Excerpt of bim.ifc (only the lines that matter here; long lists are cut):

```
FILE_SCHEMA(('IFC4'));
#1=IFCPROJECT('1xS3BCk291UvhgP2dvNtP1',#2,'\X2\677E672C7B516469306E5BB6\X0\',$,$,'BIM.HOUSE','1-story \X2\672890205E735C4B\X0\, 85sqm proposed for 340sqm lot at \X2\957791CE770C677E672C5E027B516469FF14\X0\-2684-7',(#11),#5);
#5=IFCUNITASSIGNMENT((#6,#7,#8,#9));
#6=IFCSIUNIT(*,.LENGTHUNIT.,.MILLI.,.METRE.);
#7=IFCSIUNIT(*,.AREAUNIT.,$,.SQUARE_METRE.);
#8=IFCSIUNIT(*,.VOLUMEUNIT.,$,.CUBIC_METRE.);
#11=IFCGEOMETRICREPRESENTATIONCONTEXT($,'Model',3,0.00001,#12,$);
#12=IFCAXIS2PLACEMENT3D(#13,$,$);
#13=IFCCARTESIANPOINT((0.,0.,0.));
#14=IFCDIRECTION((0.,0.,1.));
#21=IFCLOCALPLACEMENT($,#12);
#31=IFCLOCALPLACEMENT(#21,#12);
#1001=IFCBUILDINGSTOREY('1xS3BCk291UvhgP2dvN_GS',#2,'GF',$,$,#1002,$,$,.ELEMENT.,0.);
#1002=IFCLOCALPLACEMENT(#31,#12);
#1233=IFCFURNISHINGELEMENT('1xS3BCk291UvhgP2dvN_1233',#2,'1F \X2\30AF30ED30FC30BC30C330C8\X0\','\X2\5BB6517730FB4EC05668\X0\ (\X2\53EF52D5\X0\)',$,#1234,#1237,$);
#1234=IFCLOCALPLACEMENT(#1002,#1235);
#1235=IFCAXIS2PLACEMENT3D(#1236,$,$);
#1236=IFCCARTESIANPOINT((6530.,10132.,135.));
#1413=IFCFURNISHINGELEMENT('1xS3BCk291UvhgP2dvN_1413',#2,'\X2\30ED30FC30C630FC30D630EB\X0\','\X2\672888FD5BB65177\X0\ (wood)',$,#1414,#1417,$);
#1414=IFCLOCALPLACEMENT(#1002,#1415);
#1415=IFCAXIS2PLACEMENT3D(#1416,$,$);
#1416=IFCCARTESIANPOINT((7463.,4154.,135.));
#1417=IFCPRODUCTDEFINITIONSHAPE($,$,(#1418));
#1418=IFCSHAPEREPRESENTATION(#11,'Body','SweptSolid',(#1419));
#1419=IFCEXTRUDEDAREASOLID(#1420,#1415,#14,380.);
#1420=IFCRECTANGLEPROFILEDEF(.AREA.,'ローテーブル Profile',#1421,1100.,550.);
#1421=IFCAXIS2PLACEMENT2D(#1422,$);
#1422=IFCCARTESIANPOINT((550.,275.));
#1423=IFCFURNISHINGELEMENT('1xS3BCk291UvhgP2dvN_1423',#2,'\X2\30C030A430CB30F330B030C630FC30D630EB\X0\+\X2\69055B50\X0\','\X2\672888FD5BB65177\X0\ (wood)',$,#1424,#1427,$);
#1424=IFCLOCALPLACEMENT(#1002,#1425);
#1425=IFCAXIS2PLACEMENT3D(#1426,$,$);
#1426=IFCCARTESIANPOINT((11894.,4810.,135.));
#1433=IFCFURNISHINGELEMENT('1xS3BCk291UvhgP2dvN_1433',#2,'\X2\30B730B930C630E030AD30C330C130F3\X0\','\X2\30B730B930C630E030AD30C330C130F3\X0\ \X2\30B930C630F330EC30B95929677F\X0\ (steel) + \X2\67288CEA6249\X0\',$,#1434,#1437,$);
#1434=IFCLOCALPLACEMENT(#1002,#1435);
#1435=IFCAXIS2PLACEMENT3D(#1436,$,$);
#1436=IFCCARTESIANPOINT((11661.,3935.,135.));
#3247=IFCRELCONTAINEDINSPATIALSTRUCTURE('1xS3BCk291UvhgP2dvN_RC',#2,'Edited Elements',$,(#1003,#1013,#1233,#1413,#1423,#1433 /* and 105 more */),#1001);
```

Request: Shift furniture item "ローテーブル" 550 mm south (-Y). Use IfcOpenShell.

```python
import ifcopenshell
import ifcopenshell.api.geometry
import ifcopenshell.util.placement

model = ifcopenshell.open("bim.ifc")

item = model.by_id(1413)
matrix = ifcopenshell.util.placement.get_local_placement(item.ObjectPlacement)
matrix[1, 3] -= 550.0
ifcopenshell.api.geometry.edit_object_placement(model, product=item, matrix=matrix, is_si=False)

print(ifcopenshell.util.placement.get_local_placement(item.ObjectPlacement).round(3) + 0.0)

model.write("bim-out.ifc")
```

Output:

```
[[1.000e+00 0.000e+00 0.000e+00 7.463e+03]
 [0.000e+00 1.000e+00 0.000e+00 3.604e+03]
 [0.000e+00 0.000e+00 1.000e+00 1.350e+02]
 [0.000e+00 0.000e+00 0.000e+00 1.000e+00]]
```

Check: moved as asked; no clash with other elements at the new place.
